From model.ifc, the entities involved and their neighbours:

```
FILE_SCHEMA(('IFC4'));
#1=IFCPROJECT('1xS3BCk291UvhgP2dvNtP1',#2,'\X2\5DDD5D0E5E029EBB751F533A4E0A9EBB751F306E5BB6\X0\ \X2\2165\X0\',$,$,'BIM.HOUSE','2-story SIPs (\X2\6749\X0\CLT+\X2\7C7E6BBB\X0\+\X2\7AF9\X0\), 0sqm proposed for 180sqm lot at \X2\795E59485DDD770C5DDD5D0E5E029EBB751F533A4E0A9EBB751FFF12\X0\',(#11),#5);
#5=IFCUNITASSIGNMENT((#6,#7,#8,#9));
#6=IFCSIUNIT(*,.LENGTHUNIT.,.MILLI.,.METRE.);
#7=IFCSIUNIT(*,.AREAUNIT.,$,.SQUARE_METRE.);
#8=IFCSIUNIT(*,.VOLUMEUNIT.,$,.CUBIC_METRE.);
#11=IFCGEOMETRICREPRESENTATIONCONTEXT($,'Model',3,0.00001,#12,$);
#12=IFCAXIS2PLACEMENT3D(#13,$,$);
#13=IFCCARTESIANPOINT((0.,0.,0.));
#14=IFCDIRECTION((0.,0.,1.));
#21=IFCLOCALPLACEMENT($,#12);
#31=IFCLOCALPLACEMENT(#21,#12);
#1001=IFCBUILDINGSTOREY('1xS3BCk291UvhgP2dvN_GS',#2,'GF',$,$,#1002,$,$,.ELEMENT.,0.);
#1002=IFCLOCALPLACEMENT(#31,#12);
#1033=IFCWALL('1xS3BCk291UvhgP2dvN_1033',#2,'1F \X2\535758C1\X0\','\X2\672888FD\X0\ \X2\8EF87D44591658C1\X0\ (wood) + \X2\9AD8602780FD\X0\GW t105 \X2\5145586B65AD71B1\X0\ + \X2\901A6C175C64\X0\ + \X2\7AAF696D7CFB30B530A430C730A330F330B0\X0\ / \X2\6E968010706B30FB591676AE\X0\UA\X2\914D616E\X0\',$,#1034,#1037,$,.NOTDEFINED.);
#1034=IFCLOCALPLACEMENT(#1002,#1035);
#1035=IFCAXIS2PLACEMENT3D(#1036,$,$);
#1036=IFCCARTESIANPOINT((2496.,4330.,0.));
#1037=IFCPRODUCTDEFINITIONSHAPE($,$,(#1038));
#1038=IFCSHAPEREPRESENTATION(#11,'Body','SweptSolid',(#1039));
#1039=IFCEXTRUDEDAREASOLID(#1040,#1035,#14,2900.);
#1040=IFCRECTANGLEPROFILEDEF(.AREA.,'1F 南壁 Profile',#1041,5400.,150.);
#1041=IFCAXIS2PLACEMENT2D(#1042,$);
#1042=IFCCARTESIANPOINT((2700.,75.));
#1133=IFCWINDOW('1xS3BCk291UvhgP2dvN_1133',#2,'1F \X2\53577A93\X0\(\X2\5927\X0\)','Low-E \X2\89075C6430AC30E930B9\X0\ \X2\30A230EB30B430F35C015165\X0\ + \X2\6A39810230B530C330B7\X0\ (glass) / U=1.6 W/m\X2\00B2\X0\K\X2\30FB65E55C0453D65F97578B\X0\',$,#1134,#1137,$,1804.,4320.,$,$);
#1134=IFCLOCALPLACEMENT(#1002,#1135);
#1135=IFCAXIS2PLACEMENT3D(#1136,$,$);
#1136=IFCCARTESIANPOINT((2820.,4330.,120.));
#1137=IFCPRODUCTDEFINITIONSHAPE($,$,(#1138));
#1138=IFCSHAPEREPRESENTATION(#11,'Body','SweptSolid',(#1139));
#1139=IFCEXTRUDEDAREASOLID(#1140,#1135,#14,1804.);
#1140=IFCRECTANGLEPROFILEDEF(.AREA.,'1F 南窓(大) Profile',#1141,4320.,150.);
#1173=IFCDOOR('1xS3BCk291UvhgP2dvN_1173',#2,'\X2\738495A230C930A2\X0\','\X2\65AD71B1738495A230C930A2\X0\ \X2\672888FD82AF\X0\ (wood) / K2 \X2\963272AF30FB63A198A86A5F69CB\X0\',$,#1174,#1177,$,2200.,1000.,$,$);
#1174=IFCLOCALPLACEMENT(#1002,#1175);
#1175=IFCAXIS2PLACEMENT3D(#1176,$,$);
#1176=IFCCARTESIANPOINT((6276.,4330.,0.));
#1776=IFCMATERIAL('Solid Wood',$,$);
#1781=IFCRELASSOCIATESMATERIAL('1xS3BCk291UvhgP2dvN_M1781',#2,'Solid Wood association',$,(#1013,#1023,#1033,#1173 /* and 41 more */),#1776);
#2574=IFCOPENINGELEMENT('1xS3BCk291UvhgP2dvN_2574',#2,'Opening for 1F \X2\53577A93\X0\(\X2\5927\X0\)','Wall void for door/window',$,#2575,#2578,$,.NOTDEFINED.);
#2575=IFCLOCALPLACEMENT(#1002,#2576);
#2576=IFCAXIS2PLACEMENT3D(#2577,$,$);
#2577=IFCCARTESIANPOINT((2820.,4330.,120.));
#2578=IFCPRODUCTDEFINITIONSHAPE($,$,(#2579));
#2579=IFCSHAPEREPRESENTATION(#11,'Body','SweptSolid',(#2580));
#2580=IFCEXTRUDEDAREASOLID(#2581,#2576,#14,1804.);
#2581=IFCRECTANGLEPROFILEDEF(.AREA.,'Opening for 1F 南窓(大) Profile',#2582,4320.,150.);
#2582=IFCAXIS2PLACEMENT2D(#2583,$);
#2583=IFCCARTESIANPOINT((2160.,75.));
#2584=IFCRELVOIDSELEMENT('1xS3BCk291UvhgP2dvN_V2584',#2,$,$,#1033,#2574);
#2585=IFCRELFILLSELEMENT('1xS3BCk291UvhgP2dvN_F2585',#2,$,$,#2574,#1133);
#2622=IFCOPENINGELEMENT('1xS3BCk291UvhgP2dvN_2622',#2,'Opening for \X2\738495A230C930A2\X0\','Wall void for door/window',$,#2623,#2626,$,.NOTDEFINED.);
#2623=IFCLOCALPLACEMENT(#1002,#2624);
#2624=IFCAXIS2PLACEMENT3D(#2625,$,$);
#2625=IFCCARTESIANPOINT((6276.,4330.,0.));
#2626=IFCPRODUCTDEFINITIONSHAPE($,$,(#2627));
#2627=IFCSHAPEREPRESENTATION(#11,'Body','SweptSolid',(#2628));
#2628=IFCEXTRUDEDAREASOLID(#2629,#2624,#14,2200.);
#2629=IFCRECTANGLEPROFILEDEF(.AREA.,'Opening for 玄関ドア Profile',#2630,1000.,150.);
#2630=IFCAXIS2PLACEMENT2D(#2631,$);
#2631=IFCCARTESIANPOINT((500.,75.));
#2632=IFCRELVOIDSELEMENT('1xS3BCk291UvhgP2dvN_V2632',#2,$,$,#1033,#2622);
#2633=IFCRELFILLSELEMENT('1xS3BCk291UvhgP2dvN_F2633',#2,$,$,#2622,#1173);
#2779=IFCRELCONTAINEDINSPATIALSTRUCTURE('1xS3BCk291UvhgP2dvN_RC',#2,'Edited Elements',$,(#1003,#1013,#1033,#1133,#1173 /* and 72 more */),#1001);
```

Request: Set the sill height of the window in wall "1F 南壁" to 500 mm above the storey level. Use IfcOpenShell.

```python
import numpy as np
import ifcopenshell
import ifcopenshell.api.geometry
import ifcopenshell.geom
import ifcopenshell.util.element
import ifcopenshell.util.placement
import ifcopenshell.util.shape
import ifcopenshell.util.unit

model = ifcopenshell.open("model.ifc")
unit_scale = ifcopenshell.util.unit.calculate_unit_scale(model)

window = model.by_guid("1xS3BCk291UvhgP2dvN_1133")
opening = window.FillsVoids[0].RelatingOpeningElement
storey = ifcopenshell.util.element.get_container(window, ifc_class="IfcBuildingStorey")
level = ifcopenshell.util.placement.get_local_placement(storey.ObjectPlacement)[2, 3]

# The opening's origin need not be at the sill, so measure its lowest point.
shape = ifcopenshell.geom.create_shape(ifcopenshell.geom.settings(), opening)
bottom = ifcopenshell.util.shape.get_shape_bottom_elevation(shape, shape.geometry) / unit_scale
dz = level + 0.5 / unit_scale - bottom

shift = np.array([0.0, 0.0, dz])
# The window is not placed relative to its opening, so move both.
for product in (opening, window):
    matrix = ifcopenshell.util.placement.get_local_placement(product.ObjectPlacement)
    matrix[:3, 3] += shift
    ifcopenshell.api.geometry.edit_object_placement(model, product=product, matrix=matrix, is_si=False)

print(f"moved by {dz * unit_scale:+.3f} m")

model.write("model_rev.ifc")
```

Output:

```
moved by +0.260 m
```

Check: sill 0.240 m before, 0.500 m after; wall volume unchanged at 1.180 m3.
